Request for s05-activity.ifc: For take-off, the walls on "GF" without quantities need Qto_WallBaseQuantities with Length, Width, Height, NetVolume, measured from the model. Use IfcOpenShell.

First a look at what the model holds.

```python
import ifcopenshell
import ifcopenshell.util.element
import ifcopenshell.util.unit

model = ifcopenshell.open("s05-activity.ifc")
print(model.schema)
for unit_type in ("LENGTHUNIT", "AREAUNIT", "VOLUMEUNIT"):
    print(unit_type, ifcopenshell.util.unit.calculate_unit_scale(model, unit_type))
storey = next(s for s in model.by_type("IfcBuildingStorey") if s.Name == "GF")
walls = [e for e in ifcopenshell.util.element.get_decomposition(storey) if e.is_a("IfcWall")]
for e in sorted(walls, key=lambda e: e.id()):
    print(e.id(), e.is_a(), e.Name, list(ifcopenshell.util.element.get_psets(e, qtos_only=True)), sep=" | ")
```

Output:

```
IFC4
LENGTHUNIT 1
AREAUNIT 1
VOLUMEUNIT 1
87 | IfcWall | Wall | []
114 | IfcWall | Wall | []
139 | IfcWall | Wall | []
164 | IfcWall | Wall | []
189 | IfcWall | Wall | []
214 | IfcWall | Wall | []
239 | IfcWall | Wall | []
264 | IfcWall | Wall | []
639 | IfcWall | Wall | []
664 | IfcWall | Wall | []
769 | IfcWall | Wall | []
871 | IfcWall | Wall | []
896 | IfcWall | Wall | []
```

```python
import ifcopenshell
import ifcopenshell.api.pset
import ifcopenshell.geom
import ifcopenshell.util.element
import ifcopenshell.util.shape
import ifcopenshell.util.unit

model = ifcopenshell.open("s05-activity.ifc")
unit_scale = ifcopenshell.util.unit.calculate_unit_scale(model)
volume_scale = ifcopenshell.util.unit.calculate_unit_scale(model, "VOLUMEUNIT")
settings = ifcopenshell.geom.settings()

storey = next(s for s in model.by_type("IfcBuildingStorey") if s.Name == "GF")
walls = [e for e in ifcopenshell.util.element.get_decomposition(storey) if e.is_a("IfcWall")]

for e in sorted(walls, key=lambda e: e.id()):
    if ifcopenshell.util.element.get_psets(e, qtos_only=True, should_inherit=False):
        continue
    # Geometry comes back in metres, in the element's own axes.
    shape = ifcopenshell.geom.create_shape(settings, e)
    values = {
        "Length": ifcopenshell.util.shape.get_x(shape.geometry) / unit_scale,
        "Width": ifcopenshell.util.shape.get_y(shape.geometry) / unit_scale,
        "Height": ifcopenshell.util.shape.get_z(shape.geometry) / unit_scale,
        "NetVolume": ifcopenshell.util.shape.get_volume(shape.geometry) / volume_scale,
    }
    qto = ifcopenshell.api.pset.add_qto(model, product=e, name="Qto_WallBaseQuantities")
    ifcopenshell.api.pset.edit_qto(model, qto=qto, properties=values)
    print(e.id(), {k: round(v, 3) for k, v in values.items()})

model.write("s05-activity_updated.ifc")
```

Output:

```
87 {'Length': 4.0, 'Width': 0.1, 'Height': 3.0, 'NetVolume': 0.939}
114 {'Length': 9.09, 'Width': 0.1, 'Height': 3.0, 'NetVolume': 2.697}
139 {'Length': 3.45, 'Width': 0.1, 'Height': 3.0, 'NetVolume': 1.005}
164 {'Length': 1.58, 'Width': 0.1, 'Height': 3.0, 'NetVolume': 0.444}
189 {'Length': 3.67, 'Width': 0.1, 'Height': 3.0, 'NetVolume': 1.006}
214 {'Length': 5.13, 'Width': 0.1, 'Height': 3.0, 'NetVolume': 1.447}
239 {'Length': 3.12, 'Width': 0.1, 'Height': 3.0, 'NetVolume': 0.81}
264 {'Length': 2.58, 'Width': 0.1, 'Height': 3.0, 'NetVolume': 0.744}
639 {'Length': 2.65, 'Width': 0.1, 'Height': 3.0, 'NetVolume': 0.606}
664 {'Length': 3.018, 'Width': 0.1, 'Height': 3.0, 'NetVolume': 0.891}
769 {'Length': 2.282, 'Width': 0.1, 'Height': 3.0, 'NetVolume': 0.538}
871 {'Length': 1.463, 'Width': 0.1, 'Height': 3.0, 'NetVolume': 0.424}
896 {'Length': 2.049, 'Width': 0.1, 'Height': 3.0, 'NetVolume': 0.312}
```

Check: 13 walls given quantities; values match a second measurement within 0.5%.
